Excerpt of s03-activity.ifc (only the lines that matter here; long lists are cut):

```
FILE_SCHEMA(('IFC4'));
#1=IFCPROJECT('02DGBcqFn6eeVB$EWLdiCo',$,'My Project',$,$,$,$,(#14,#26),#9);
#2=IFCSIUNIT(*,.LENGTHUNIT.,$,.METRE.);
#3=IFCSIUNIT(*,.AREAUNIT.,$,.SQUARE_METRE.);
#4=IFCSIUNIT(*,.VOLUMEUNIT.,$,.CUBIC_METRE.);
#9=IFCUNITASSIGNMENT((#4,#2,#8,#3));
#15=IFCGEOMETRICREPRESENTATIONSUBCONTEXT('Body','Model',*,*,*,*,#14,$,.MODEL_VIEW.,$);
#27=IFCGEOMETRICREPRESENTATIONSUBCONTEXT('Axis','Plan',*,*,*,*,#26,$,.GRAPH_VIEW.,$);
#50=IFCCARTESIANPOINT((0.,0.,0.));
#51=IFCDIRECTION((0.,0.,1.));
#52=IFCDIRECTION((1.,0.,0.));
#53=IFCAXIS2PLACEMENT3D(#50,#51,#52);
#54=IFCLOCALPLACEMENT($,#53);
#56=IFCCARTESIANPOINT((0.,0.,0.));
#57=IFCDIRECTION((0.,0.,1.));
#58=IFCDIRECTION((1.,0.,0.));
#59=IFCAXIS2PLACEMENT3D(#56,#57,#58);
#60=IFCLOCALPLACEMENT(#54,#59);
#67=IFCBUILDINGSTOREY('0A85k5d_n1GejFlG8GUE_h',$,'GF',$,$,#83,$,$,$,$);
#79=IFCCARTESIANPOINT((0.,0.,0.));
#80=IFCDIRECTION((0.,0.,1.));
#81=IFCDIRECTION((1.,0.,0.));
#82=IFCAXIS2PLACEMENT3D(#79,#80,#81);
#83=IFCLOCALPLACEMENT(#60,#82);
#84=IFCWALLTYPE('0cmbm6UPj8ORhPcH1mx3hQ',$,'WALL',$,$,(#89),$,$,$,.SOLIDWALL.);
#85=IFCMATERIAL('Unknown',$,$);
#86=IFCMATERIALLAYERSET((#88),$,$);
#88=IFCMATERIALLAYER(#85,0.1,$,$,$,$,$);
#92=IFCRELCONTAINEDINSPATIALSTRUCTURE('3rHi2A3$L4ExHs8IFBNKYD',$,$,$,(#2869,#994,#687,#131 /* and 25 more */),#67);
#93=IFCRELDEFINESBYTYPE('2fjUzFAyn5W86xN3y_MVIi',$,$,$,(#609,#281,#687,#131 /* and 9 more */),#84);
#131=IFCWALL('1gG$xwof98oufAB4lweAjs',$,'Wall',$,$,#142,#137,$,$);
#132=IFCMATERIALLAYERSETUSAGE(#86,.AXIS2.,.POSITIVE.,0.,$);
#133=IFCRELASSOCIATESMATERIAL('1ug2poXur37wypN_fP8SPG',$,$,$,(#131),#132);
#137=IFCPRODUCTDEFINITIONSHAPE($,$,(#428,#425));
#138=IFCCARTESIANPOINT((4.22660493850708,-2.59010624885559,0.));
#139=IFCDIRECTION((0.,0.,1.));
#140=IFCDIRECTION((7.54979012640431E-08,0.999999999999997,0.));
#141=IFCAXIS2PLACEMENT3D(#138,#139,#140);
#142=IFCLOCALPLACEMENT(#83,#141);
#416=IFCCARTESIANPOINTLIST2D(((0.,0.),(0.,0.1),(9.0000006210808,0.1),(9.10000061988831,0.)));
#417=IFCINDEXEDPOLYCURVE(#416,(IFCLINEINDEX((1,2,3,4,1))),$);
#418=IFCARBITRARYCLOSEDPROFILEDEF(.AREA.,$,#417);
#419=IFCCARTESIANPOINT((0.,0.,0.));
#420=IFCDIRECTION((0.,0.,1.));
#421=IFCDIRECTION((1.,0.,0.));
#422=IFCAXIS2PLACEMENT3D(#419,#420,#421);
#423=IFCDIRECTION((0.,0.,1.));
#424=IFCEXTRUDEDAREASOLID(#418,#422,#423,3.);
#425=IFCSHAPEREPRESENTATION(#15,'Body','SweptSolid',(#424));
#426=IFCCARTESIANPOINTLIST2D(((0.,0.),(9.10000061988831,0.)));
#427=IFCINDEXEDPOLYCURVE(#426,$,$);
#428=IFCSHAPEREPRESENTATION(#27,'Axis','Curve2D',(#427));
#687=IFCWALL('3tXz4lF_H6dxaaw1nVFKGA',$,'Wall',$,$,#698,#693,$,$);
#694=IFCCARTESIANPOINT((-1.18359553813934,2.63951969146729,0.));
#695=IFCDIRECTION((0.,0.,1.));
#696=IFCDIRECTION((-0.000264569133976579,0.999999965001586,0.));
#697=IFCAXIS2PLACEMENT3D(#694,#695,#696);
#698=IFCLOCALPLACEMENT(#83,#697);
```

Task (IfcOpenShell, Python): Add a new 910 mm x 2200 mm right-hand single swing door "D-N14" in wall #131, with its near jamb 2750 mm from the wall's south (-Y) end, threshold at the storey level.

```python
import numpy as np
import ifcopenshell
import ifcopenshell.api.feature
import ifcopenshell.api.geometry
import ifcopenshell.api.root
import ifcopenshell.api.spatial
import ifcopenshell.geom
import ifcopenshell.util.element
import ifcopenshell.util.placement
import ifcopenshell.util.representation
import ifcopenshell.util.shape
import ifcopenshell.util.unit

model = ifcopenshell.open("s03-activity.ifc")
unit_scale = ifcopenshell.util.unit.calculate_unit_scale(model)
settings = ifcopenshell.geom.settings()


def volume(element):
    """Net volume in cubic metres, openings subtracted."""
    shape = ifcopenshell.geom.create_shape(settings, element)
    return ifcopenshell.util.shape.get_volume(shape.geometry)


wall = model.by_id(131)
storey = ifcopenshell.util.element.get_container(wall, ifc_class="IfcBuildingStorey")
context = ifcopenshell.util.representation.get_context(model, "Model", "Body", "MODEL_VIEW")
before = volume(wall)

width, height, from_end, sill = 0.91, 2.2, 2.75, 0.0  # metres

# The wall runs along its own X axis, and the end named is its -X end.
wall_shape = ifcopenshell.geom.create_shape(settings, wall)
x, y, z = ifcopenshell.util.shape.get_vertices(wall_shape.geometry).T
start = x.min() + from_end
face, thickness = float(y.min()), float(y.max() - y.min())
wall_matrix = ifcopenshell.util.placement.get_local_placement(wall.ObjectPlacement)
level = ifcopenshell.util.placement.get_local_placement(storey.ObjectPlacement)[2, 3]


def in_wall(x, y):
    """Placement at x, y metres in the wall's axes, at sill height."""
    matrix = wall_matrix.copy()
    matrix[:, 3] = wall_matrix @ np.array([x / unit_scale, y / unit_scale, 0.0, 1.0])
    matrix[2, 3] = level + sill / unit_scale
    return matrix


# Opening: a box that overshoots both wall faces by 50 mm.
opening = ifcopenshell.api.root.create_entity(model, ifc_class="IfcOpeningElement", predefined_type="OPENING")
box = ifcopenshell.api.geometry.add_wall_representation(
    model, context=context, length=width, height=height, thickness=thickness + 0.1
)
ifcopenshell.api.geometry.assign_representation(model, product=opening, representation=box)
ifcopenshell.api.geometry.edit_object_placement(model, product=opening, matrix=in_wall(start, face - 0.05), is_si=False)
ifcopenshell.api.feature.add_feature(model, feature=opening, element=wall)

door = ifcopenshell.api.root.create_entity(model, ifc_class="IfcDoor", name="D-N14", predefined_type="DOOR")
door.OverallWidth, door.OverallHeight = width / unit_scale, height / unit_scale
door.OperationType = "SINGLE_SWING_RIGHT"
body = ifcopenshell.api.geometry.add_door_representation(
    model,
    context=context,
    overall_width=door.OverallWidth,
    overall_height=door.OverallHeight,
    operation_type="SINGLE_SWING_RIGHT",
    lining_properties={"LiningDepth": thickness / unit_scale, "ThresholdDepth": thickness / unit_scale},
)
ifcopenshell.api.geometry.assign_representation(model, product=door, representation=body)
ifcopenshell.api.spatial.assign_container(model, products=[door], relating_structure=storey)
ifcopenshell.api.feature.add_filling(model, opening=opening, element=door)

# The lining spans the wall, so the door starts at the wall face.
ifcopenshell.api.geometry.edit_object_placement(model, product=door, matrix=in_wall(start, face), is_si=False)

after = volume(wall)

print(f"wall volume {before:.3f} -> {after:.3f} m3")

model.write("s03-activity_updated.ifc")
```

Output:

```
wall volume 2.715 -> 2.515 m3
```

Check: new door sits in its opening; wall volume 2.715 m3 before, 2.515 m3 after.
